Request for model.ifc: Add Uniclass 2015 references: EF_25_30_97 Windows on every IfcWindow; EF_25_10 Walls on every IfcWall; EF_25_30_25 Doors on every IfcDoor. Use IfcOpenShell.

First a look at what the model holds.

```python
import ifcopenshell

model = ifcopenshell.open("model.ifc")
print(model.schema)
print("classifications:", [c.Name for c in model.by_type("IfcClassification")])
for ifc_class in ("IfcDoor", "IfcRoof", "IfcStair", "IfcWall", "IfcWindow"):
    print(ifc_class, len(model.by_type(ifc_class)))
```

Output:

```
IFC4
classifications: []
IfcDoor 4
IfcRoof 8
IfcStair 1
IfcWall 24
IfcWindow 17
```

```python
import ifcopenshell
import ifcopenshell.api.classification

model = ifcopenshell.open("model.ifc")

system = ifcopenshell.api.classification.add_classification(model, classification="Uniclass 2015")

codes = {
    "IfcWindow": ("EF_25_30_97", "Windows"),
    "IfcWall": ("EF_25_10", "Walls"),
    "IfcDoor": ("EF_25_30_25", "Doors"),
}
for ifc_class, (code, name) in codes.items():
    products = model.by_type(ifc_class)
    ifcopenshell.api.classification.add_reference(
        model, products=products, classification=system, identification=code, name=name
    )
    print(code, len(products))

model.write("model_rev.ifc")
```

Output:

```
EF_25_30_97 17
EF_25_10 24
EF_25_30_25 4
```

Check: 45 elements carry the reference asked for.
